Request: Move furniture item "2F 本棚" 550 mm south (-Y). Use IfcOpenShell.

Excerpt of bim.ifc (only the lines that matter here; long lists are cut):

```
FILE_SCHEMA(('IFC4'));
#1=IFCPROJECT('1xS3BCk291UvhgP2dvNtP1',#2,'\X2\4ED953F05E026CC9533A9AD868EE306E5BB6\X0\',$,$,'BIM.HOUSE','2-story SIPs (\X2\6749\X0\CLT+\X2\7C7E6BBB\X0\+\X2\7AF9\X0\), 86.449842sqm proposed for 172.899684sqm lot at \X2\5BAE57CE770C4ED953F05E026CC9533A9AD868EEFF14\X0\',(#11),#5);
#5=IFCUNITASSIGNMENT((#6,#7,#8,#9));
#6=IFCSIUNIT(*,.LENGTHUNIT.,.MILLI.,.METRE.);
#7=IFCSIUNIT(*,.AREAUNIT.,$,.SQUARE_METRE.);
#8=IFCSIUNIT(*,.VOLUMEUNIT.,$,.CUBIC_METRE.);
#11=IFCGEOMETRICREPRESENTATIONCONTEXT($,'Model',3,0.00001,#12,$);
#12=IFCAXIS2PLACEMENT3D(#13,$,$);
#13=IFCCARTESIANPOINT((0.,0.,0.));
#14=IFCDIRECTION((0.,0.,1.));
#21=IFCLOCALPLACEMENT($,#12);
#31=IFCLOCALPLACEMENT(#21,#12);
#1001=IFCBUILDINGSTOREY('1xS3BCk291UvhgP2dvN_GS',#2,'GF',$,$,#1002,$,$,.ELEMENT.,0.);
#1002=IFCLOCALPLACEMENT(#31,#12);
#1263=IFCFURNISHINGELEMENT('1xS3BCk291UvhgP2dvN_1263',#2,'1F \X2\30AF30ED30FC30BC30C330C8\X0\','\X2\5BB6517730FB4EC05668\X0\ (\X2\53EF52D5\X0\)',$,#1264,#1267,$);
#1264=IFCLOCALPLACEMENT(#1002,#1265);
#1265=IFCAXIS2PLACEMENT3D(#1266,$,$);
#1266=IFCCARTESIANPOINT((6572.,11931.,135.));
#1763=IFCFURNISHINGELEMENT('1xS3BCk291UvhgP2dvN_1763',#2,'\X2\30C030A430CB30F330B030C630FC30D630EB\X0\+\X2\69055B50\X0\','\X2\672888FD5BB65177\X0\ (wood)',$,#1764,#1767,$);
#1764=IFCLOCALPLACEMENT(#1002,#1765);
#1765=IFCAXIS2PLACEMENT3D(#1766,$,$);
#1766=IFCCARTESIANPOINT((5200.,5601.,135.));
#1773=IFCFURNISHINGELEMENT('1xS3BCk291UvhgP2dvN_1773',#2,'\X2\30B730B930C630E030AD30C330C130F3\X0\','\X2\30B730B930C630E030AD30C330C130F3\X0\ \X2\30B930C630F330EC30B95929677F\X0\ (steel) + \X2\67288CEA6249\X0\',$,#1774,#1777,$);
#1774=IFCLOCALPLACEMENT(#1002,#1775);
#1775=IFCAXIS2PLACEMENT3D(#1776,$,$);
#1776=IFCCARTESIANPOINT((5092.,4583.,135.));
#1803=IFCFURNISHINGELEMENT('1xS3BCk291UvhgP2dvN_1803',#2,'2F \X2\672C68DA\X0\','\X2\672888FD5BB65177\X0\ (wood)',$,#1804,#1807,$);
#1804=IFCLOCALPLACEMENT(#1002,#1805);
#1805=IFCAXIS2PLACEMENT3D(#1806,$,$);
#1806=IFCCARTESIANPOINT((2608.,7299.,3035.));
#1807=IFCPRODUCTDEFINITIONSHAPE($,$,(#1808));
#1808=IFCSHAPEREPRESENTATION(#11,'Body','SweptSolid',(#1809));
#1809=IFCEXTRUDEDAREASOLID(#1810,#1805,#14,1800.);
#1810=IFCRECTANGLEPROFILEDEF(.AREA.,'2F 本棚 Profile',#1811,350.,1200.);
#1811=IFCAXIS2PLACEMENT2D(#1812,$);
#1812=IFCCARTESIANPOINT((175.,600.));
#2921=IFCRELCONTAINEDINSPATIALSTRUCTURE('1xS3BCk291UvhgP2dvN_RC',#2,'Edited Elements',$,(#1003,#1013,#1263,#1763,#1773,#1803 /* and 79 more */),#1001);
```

```python
import ifcopenshell
import ifcopenshell.api.geometry
import ifcopenshell.util.placement
import ifcopenshell.util.unit

model = ifcopenshell.open("bim.ifc")
unit_scale = ifcopenshell.util.unit.calculate_unit_scale(model)

item = model.by_guid("1xS3BCk291UvhgP2dvN_1803")
matrix = ifcopenshell.util.placement.get_local_placement(item.ObjectPlacement)
matrix[1, 3] -= 0.55 / unit_scale
ifcopenshell.api.geometry.edit_object_placement(model, product=item, matrix=matrix, is_si=False)

print(ifcopenshell.util.placement.get_local_placement(item.ObjectPlacement).round(3) + 0.0)

model.write("bim_rev.ifc")
```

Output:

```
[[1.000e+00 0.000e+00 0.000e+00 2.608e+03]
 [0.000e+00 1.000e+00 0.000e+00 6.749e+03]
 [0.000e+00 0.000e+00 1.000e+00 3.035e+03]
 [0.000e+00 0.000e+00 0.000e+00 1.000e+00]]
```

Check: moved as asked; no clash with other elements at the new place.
